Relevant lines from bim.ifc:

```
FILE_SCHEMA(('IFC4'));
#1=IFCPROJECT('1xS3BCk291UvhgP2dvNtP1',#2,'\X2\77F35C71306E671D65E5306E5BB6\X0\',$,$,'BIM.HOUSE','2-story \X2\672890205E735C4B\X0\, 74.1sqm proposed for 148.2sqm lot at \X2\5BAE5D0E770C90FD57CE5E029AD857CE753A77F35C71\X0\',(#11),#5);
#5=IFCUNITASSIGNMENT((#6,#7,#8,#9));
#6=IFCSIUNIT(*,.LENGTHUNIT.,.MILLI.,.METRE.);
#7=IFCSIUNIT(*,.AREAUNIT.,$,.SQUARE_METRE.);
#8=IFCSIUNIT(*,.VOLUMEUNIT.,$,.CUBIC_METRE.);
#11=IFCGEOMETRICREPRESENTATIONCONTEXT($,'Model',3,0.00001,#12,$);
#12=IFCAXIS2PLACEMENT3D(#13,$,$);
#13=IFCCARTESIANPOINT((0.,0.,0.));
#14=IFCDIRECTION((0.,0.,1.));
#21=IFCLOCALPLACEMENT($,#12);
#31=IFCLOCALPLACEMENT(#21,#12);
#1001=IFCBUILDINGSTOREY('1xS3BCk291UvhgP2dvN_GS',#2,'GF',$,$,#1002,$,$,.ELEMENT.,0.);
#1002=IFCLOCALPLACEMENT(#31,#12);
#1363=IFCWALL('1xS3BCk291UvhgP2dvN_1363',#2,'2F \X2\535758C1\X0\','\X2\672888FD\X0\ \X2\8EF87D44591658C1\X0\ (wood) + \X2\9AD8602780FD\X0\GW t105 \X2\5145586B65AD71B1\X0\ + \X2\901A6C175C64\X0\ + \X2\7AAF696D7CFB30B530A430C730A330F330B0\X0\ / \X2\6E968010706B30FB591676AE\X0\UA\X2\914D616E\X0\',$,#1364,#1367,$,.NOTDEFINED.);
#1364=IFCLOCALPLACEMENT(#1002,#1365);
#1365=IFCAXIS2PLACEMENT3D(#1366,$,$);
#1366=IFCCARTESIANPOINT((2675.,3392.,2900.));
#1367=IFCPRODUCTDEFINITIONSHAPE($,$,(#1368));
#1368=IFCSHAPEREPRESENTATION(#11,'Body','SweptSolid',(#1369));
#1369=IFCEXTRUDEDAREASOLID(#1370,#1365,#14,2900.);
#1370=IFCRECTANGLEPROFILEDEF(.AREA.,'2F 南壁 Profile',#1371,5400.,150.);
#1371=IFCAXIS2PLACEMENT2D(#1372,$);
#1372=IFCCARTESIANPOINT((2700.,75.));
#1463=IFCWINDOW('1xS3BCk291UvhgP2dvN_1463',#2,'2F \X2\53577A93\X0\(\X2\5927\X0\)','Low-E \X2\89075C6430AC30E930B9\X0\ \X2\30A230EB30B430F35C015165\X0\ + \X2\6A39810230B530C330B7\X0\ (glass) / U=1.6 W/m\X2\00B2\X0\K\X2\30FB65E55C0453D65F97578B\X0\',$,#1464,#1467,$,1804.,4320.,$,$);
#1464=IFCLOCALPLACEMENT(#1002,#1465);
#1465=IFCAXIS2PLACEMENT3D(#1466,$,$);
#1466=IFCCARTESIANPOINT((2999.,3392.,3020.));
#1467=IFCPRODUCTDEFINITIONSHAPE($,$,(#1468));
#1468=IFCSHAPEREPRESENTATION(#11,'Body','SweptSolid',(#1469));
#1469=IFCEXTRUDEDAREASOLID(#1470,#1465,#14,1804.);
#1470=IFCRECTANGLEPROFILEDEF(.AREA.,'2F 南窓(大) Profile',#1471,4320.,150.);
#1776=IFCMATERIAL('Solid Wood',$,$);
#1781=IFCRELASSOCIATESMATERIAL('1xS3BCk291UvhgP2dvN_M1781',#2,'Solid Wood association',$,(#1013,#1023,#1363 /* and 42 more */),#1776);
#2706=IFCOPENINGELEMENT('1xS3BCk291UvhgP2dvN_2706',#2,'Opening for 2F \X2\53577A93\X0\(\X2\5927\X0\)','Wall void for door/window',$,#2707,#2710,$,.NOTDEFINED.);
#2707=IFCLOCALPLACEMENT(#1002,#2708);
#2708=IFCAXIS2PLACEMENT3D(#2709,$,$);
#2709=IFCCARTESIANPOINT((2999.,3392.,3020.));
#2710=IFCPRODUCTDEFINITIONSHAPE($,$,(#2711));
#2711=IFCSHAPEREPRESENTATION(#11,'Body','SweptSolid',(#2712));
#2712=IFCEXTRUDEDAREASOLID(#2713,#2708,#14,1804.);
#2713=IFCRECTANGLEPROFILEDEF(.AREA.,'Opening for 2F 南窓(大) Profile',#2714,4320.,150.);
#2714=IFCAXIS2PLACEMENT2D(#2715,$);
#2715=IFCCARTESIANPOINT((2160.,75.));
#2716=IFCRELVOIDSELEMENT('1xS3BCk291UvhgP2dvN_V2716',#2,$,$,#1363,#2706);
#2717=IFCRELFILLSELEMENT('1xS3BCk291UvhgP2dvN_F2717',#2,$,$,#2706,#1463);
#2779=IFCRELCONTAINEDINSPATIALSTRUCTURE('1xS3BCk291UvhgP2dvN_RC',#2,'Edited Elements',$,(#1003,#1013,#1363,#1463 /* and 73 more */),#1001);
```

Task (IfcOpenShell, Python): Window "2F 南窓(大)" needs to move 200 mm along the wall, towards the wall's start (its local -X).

```python
import ifcopenshell
import ifcopenshell.api.geometry
import ifcopenshell.util.placement
import ifcopenshell.util.unit

model = ifcopenshell.open("bim.ifc")
unit_scale = ifcopenshell.util.unit.calculate_unit_scale(model)

window = model.by_guid("1xS3BCk291UvhgP2dvN_1463")
opening = window.FillsVoids[0].RelatingOpeningElement
wall = opening.VoidsElements[0].RelatingBuildingElement

wall_matrix = ifcopenshell.util.placement.get_local_placement(wall.ObjectPlacement)
shift = wall_matrix[:3, 0] * -0.2 / unit_scale
before = ifcopenshell.util.placement.get_local_placement(window.ObjectPlacement)[:3, 3].copy()

# The window is not placed relative to its opening, so move both.
for product in (opening, window):
    matrix = ifcopenshell.util.placement.get_local_placement(product.ObjectPlacement)
    matrix[:3, 3] += shift
    ifcopenshell.api.geometry.edit_object_placement(model, product=product, matrix=matrix, is_si=False)

after = ifcopenshell.util.placement.get_local_placement(window.ObjectPlacement)[:3, 3]
print("window moved by", (after - before).round(3) + 0.0)

model.write("bim_updated.ifc")
```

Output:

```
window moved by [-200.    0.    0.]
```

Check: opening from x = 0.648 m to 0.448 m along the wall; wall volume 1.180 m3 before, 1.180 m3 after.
